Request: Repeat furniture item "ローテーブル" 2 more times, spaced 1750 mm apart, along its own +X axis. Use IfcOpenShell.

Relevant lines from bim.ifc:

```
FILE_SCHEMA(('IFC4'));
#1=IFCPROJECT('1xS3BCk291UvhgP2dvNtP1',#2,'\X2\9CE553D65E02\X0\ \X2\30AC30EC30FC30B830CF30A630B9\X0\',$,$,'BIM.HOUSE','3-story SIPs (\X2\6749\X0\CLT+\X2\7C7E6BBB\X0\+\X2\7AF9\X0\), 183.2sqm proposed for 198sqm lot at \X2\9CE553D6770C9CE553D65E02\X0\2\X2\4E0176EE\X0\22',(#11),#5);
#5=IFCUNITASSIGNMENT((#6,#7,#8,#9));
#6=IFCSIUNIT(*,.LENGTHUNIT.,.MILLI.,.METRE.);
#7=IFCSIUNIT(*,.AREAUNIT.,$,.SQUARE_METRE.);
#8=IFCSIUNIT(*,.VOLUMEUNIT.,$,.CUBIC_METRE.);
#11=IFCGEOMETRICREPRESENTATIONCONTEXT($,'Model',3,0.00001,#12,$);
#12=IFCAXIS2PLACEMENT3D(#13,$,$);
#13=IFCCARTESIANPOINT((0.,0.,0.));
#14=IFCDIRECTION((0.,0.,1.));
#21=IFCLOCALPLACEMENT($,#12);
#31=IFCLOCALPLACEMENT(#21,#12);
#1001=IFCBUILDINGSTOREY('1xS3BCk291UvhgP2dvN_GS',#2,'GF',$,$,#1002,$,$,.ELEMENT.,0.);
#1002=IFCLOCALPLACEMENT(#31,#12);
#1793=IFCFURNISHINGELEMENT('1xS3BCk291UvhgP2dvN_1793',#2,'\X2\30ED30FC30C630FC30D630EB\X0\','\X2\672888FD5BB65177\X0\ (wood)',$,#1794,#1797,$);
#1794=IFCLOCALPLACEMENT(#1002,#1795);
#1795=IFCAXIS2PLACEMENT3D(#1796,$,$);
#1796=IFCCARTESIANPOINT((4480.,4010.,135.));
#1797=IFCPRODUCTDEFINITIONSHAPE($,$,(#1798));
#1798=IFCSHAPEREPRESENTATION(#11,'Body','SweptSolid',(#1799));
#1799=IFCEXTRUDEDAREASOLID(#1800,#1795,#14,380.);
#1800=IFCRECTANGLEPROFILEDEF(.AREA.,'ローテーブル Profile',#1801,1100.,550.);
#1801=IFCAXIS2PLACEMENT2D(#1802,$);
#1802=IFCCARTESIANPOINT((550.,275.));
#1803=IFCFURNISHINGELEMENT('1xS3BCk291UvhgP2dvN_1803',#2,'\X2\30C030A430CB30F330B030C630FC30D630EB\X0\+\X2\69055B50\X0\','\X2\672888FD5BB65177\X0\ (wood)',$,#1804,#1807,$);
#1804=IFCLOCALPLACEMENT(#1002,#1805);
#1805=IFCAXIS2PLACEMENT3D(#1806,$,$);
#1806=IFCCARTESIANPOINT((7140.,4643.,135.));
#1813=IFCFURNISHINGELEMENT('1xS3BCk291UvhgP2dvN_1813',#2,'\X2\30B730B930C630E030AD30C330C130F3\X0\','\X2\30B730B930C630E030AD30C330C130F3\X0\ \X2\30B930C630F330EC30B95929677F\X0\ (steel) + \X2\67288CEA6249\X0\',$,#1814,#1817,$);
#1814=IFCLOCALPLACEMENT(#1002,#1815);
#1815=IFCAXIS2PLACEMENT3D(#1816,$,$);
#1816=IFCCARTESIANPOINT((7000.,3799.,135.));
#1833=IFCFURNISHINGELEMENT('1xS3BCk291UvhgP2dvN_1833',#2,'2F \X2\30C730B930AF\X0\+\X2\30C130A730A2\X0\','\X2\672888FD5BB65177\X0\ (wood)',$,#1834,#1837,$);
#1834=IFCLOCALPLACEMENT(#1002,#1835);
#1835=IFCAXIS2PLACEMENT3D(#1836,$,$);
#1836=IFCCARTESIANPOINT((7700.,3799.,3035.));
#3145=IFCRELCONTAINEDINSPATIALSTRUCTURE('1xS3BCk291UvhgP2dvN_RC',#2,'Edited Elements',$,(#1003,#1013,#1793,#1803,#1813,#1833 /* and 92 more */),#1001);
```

```python
import ifcopenshell
import ifcopenshell.api.geometry
import ifcopenshell.api.root
import ifcopenshell.util.element
import ifcopenshell.util.placement
import ifcopenshell.util.unit

model = ifcopenshell.open("bim.ifc")
unit_scale = ifcopenshell.util.unit.calculate_unit_scale(model)


def reuse_history(source, copy):
    """copy_class also copies each property set's owner history, people and application; keep the originals."""
    for rel in copy.IsDefinedBy:
        if rel.is_a("IfcRelDefinesByProperties") and (history := rel.RelatingPropertyDefinition.OwnerHistory):
            rel.RelatingPropertyDefinition.OwnerHistory = source.OwnerHistory
            ifcopenshell.util.element.remove_deep2(model, history)


source = model.by_guid("1xS3BCk291UvhgP2dvN_1793")
base = ifcopenshell.util.placement.get_local_placement(source.ObjectPlacement)
step = base[:3, 0] * 1.75 / unit_scale

for i in range(1, 3):
    copy = ifcopenshell.api.root.copy_class(model, product=source)
    copy.Representation = ifcopenshell.util.element.copy_deep(
        model, source.Representation, exclude=["IfcGeometricRepresentationContext", "IfcRepresentationMap"]
    )
    reuse_history(source, copy)
    matrix = base.copy()
    matrix[:3, 3] += i * step
    print("added at", matrix[:3, 3].round(3) + 0.0)
    ifcopenshell.api.geometry.edit_object_placement(model, product=copy, matrix=matrix, is_si=False)

model.write("bim_updated.ifc")
```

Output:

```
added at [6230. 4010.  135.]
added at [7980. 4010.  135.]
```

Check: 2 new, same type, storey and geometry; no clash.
